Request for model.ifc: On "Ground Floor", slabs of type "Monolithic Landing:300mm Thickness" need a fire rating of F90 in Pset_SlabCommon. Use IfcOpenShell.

First a look at what the model holds.

```python
import ifcopenshell
import ifcopenshell.util.element

model = ifcopenshell.open("model.ifc")
print(model.schema)
storey = next(s for s in model.by_type("IfcBuildingStorey") if s.Name == "Ground Floor")
slabs = [e for e in ifcopenshell.util.element.get_decomposition(storey) if e.is_a("IfcSlab")]
seen = {}
for e in slabs:
    element_type = ifcopenshell.util.element.get_type(e)
    key = (element_type.Name if element_type != e and element_type else None, ifcopenshell.util.element.get_pset(e, "Pset_SlabCommon", "FireRating"))
    seen[key] = seen.get(key, 0) + 1
for (name, value), count in sorted(seen.items(), key=str):
    print(count, "x", name, "|", value)
```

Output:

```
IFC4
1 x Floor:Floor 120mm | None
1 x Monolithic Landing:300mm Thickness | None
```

```python
import ifcopenshell
import ifcopenshell.api.pset
import ifcopenshell.util.element

model = ifcopenshell.open("model.ifc")

storey = next(s for s in model.by_type("IfcBuildingStorey") if s.Name == "Ground Floor")
slabs = [e for e in ifcopenshell.util.element.get_decomposition(storey) if e.is_a("IfcSlab")]

count = 0
for e in slabs:
    element_type = ifcopenshell.util.element.get_type(e)
    if element_type in (None, e) or element_type.Name != "Monolithic Landing:300mm Thickness":
        continue
    # add_pset returns the element's existing set when there is one.
    pset = ifcopenshell.api.pset.add_pset(model, product=e, name="Pset_SlabCommon")
    ifcopenshell.api.pset.edit_pset(model, pset=pset, properties={"FireRating": "F90"})
    count += 1

print(count, "slabs updated")

model.write("model_v2.ifc")
```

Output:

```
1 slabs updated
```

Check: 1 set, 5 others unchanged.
